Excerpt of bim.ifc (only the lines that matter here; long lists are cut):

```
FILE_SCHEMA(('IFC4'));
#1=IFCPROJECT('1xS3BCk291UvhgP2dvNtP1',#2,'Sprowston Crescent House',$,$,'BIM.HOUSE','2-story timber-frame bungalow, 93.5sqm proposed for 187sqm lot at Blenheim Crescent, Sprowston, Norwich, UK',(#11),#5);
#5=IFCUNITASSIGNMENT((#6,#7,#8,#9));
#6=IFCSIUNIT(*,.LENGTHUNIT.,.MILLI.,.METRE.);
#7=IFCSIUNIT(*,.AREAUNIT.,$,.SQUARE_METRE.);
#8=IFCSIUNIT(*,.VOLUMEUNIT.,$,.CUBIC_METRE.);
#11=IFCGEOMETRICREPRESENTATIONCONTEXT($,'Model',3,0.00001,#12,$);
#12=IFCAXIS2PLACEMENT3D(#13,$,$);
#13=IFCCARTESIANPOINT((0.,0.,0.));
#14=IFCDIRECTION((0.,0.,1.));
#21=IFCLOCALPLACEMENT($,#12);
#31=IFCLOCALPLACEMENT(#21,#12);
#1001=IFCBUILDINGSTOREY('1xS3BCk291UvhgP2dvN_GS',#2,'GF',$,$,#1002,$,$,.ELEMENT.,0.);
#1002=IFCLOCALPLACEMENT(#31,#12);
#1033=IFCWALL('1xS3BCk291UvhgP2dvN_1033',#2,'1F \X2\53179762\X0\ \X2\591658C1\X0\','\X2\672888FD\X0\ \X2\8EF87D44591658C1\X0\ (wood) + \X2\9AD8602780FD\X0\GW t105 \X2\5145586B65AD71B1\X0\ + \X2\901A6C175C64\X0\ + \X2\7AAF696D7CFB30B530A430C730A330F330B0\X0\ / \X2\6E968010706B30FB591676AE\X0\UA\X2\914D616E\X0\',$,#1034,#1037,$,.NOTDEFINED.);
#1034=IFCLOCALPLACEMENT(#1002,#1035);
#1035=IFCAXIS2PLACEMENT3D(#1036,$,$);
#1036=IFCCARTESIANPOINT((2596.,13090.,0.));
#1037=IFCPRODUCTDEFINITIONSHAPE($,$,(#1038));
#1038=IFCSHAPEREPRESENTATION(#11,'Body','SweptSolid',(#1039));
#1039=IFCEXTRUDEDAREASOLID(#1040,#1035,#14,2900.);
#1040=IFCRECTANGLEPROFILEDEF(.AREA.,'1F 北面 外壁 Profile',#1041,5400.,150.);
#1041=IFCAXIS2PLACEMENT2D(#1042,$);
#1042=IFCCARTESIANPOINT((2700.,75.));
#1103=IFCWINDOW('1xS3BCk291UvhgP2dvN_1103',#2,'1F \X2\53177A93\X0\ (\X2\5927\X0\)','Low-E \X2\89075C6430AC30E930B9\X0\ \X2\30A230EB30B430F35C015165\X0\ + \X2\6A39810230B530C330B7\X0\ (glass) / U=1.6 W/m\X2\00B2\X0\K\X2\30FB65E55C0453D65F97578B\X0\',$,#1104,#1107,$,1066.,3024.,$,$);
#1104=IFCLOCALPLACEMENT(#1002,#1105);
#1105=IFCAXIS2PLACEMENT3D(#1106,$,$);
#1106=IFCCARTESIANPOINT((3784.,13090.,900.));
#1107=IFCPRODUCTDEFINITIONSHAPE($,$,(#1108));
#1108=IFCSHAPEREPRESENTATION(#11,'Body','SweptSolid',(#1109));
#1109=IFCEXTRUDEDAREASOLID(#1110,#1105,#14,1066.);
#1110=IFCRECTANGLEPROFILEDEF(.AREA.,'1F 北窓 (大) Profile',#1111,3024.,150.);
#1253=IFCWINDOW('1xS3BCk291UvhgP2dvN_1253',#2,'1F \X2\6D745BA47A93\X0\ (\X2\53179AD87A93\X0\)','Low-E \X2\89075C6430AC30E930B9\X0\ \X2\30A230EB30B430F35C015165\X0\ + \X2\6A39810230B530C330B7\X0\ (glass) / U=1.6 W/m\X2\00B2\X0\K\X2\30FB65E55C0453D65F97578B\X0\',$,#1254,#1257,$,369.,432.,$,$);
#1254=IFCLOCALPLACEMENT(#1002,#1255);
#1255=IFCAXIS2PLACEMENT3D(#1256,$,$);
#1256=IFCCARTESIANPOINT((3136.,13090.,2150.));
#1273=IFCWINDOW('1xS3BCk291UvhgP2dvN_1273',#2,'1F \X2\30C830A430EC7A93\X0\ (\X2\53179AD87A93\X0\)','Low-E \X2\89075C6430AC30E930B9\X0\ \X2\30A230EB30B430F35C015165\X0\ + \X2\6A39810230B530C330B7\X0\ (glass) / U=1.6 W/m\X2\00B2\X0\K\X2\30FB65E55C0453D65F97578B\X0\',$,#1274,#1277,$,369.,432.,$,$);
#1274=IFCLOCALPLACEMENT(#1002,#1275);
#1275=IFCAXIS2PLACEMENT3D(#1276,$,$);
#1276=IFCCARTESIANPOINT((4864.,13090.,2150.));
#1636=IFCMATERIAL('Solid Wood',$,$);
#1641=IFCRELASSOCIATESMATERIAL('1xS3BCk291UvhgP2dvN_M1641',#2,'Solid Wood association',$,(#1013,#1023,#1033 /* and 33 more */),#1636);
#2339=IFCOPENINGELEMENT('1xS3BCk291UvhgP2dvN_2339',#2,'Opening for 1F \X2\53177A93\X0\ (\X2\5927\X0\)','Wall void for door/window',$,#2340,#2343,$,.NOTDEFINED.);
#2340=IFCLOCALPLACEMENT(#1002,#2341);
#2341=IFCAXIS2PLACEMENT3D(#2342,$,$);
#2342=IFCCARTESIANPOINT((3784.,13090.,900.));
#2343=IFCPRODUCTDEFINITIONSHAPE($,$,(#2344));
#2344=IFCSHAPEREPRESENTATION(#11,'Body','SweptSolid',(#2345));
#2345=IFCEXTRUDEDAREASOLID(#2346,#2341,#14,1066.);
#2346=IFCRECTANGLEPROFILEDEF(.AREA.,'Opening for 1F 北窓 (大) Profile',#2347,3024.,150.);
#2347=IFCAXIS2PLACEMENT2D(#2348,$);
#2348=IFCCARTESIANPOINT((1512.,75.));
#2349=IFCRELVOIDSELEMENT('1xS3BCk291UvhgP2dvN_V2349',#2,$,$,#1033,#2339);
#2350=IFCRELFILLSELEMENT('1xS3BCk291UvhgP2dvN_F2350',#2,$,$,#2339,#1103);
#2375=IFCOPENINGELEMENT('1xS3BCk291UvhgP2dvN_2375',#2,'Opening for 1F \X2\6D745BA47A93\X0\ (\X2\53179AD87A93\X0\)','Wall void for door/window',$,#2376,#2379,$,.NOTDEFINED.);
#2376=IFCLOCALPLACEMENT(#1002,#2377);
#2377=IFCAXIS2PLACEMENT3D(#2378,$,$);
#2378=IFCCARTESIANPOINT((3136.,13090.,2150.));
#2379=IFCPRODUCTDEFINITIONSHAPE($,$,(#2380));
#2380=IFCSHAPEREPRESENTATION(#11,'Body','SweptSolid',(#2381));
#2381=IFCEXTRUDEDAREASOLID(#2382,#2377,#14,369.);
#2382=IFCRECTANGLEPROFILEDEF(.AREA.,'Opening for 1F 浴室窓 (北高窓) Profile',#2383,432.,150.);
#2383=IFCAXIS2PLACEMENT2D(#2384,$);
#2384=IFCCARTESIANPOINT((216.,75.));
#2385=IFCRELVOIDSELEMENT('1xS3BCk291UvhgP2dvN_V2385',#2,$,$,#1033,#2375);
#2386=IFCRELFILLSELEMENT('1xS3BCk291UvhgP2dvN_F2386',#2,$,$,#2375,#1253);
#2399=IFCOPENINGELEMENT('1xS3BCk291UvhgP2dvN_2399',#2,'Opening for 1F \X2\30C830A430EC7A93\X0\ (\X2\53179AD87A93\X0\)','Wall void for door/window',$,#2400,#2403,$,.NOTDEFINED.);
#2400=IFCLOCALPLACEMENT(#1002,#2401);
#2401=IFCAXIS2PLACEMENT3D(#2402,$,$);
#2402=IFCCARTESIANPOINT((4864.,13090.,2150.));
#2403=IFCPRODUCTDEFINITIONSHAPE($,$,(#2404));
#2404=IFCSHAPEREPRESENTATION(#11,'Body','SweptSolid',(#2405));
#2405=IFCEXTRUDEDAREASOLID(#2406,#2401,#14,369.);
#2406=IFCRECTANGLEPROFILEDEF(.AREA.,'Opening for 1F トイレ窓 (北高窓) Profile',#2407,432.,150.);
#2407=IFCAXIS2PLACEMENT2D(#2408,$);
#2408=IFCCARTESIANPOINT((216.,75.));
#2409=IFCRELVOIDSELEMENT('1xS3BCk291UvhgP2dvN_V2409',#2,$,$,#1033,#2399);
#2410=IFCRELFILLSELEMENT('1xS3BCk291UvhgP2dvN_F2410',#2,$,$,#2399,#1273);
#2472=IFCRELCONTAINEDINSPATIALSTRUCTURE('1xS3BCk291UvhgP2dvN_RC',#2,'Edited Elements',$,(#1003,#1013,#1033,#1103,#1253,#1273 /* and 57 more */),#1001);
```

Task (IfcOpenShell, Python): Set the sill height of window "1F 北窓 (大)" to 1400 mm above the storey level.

```python
import numpy as np
import ifcopenshell
import ifcopenshell.api.geometry
import ifcopenshell.geom
import ifcopenshell.util.element
import ifcopenshell.util.placement
import ifcopenshell.util.shape
import ifcopenshell.util.unit

model = ifcopenshell.open("bim.ifc")
unit_scale = ifcopenshell.util.unit.calculate_unit_scale(model)

window = model.by_guid("1xS3BCk291UvhgP2dvN_1103")
opening = window.FillsVoids[0].RelatingOpeningElement
storey = ifcopenshell.util.element.get_container(window, ifc_class="IfcBuildingStorey")
level = ifcopenshell.util.placement.get_local_placement(storey.ObjectPlacement)[2, 3]

# The opening's origin need not be at the sill, so measure its lowest point.
shape = ifcopenshell.geom.create_shape(ifcopenshell.geom.settings(), opening)
bottom = ifcopenshell.util.shape.get_shape_bottom_elevation(shape, shape.geometry) / unit_scale
dz = level + 1400.0 - bottom

shift = np.array([0.0, 0.0, dz])
# The window is not placed relative to its opening, so move both.
for product in (opening, window):
    matrix = ifcopenshell.util.placement.get_local_placement(product.ObjectPlacement)
    matrix[:3, 3] += shift
    ifcopenshell.api.geometry.edit_object_placement(model, product=product, matrix=matrix, is_si=False)

print(f"moved by {dz * unit_scale:+.3f} m")

model.write("bim-out.ifc")
```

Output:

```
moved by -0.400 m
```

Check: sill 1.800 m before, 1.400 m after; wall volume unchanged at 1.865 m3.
